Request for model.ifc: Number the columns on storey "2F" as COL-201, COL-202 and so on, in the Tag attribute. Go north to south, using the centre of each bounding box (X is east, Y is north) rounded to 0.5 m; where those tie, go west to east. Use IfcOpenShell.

First a look at what the model holds.

```python
import ifcopenshell
import ifcopenshell.util.element
import ifcopenshell.util.placement

model = ifcopenshell.open("model.ifc")
print(model.schema)
storey = next(s for s in model.by_type("IfcBuildingStorey") if s.Name == "2F")
columns = [e for e in ifcopenshell.util.element.get_decomposition(storey) if e.is_a("IfcColumn")]
for e in sorted(columns, key=lambda e: e.id()):
    origin = ifcopenshell.util.placement.get_local_placement(e.ObjectPlacement)[:3, 3]
    print(e.id(), e.Tag, e.Name, origin.round(2) + 0.0, sep=" | ")
```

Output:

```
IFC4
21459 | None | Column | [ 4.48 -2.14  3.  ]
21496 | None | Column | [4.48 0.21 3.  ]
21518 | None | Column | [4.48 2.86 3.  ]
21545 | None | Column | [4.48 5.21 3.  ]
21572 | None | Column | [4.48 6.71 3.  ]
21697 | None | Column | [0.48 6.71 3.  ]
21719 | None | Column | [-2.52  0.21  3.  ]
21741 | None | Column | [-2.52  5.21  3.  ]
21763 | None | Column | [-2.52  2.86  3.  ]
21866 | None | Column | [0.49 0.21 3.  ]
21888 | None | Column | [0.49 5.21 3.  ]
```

```python
import ifcopenshell
import ifcopenshell.geom
import ifcopenshell.util.element
import ifcopenshell.util.shape

model = ifcopenshell.open("model.ifc")
settings = ifcopenshell.geom.settings()
settings.set("use-world-coords", True)


def centre(element):
    shape = ifcopenshell.geom.create_shape(settings, element)
    return ifcopenshell.util.shape.get_bbox_centroid(shape.geometry)


storey = next(s for s in model.by_type("IfcBuildingStorey") if s.Name == "2F")
columns = [e for e in ifcopenshell.util.element.get_decomposition(storey) if e.is_a("IfcColumn")]

# Insertion points can sit at a corner or the storey origin, so sort by the geometry (in metres).
centres = {e: centre(e) for e in columns}
columns.sort(key=lambda e: (-round(centres[e][1] / 0.5), centres[e][0]))

for i, e in enumerate(columns, start=1):
    number = f"COL-2{i:02d}"
    e.Tag = number
    print(e.id(), number)

model.write("model_updated.ifc")
```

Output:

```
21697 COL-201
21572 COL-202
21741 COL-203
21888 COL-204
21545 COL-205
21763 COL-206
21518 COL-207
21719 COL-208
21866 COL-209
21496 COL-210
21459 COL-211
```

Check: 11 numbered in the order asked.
